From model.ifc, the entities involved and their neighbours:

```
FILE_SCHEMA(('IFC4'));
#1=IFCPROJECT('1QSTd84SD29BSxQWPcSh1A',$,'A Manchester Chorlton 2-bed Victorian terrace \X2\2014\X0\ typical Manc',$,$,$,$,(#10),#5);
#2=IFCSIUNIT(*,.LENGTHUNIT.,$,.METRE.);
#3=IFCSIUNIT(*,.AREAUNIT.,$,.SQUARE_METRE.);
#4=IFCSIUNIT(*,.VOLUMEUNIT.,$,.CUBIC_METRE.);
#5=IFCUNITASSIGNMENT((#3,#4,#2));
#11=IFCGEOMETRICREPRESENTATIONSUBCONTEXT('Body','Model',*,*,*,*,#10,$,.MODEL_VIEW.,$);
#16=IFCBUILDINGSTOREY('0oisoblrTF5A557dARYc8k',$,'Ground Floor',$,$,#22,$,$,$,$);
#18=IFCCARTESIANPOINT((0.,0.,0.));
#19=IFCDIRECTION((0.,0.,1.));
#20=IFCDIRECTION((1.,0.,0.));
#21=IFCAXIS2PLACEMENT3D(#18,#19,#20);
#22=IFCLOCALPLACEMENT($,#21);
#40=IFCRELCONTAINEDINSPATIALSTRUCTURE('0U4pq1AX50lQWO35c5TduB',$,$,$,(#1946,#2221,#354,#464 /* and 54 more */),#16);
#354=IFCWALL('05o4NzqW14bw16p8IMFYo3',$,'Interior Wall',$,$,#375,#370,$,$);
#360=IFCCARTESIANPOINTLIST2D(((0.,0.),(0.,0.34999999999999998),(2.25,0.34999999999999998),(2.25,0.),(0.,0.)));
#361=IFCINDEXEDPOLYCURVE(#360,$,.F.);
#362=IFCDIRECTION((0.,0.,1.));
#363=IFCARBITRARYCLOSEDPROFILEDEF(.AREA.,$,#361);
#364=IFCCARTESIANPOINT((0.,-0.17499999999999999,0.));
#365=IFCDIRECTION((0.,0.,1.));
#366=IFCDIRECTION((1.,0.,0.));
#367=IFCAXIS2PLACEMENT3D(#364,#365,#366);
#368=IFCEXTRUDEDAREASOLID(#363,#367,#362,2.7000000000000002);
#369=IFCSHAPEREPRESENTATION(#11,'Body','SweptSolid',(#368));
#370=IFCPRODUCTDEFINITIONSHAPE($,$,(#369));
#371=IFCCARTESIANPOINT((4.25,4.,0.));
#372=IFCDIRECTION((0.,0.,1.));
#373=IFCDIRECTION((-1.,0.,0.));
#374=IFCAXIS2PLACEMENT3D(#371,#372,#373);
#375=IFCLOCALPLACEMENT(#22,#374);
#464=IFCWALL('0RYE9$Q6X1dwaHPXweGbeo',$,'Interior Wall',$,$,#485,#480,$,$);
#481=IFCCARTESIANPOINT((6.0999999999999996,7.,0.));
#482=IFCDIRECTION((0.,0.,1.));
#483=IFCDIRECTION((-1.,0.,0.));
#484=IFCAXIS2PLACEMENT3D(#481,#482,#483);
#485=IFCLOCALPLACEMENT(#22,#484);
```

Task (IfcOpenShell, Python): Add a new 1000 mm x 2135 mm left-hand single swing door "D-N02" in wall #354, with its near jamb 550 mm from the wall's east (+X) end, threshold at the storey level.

```python
import numpy as np
import ifcopenshell
import ifcopenshell.api.feature
import ifcopenshell.api.geometry
import ifcopenshell.api.root
import ifcopenshell.api.spatial
import ifcopenshell.geom
import ifcopenshell.util.element
import ifcopenshell.util.placement
import ifcopenshell.util.representation
import ifcopenshell.util.shape
import ifcopenshell.util.unit

model = ifcopenshell.open("model.ifc")
unit_scale = ifcopenshell.util.unit.calculate_unit_scale(model)
settings = ifcopenshell.geom.settings()


def volume(element):
    """Net volume in cubic metres, openings subtracted."""
    shape = ifcopenshell.geom.create_shape(settings, element)
    return ifcopenshell.util.shape.get_volume(shape.geometry)


wall = model.by_id(354)
storey = ifcopenshell.util.element.get_container(wall, ifc_class="IfcBuildingStorey")
context = ifcopenshell.util.representation.get_context(model, "Model", "Body", "MODEL_VIEW")
before = volume(wall)

width, height, from_end, sill = 1, 2.135, 0.55, 0.0  # metres

# The wall runs along its own X axis, and the end named is its -X end.
wall_shape = ifcopenshell.geom.create_shape(settings, wall)
x, y, z = ifcopenshell.util.shape.get_vertices(wall_shape.geometry).T
start = x.min() + from_end
face, thickness = float(y.min()), float(y.max() - y.min())
wall_matrix = ifcopenshell.util.placement.get_local_placement(wall.ObjectPlacement)
level = ifcopenshell.util.placement.get_local_placement(storey.ObjectPlacement)[2, 3]


def in_wall(x, y):
    """Placement at x, y metres in the wall's axes, at sill height."""
    matrix = wall_matrix.copy()
    matrix[:, 3] = wall_matrix @ np.array([x / unit_scale, y / unit_scale, 0.0, 1.0])
    matrix[2, 3] = level + sill / unit_scale
    return matrix


# Opening: a box that overshoots both wall faces by 50 mm.
opening = ifcopenshell.api.root.create_entity(model, ifc_class="IfcOpeningElement", predefined_type="OPENING")
box = ifcopenshell.api.geometry.add_wall_representation(
    model, context=context, length=width, height=height, thickness=thickness + 0.1
)
ifcopenshell.api.geometry.assign_representation(model, product=opening, representation=box)
ifcopenshell.api.geometry.edit_object_placement(model, product=opening, matrix=in_wall(start, face - 0.05), is_si=False)
ifcopenshell.api.feature.add_feature(model, feature=opening, element=wall)

door = ifcopenshell.api.root.create_entity(model, ifc_class="IfcDoor", name="D-N02", predefined_type="DOOR")
door.OverallWidth, door.OverallHeight = width / unit_scale, height / unit_scale
door.OperationType = "SINGLE_SWING_LEFT"
body = ifcopenshell.api.geometry.add_door_representation(
    model,
    context=context,
    overall_width=door.OverallWidth,
    overall_height=door.OverallHeight,
    operation_type="SINGLE_SWING_LEFT",
    lining_properties={"LiningDepth": thickness / unit_scale, "ThresholdDepth": thickness / unit_scale},
)
ifcopenshell.api.geometry.assign_representation(model, product=door, representation=body)
ifcopenshell.api.spatial.assign_container(model, products=[door], relating_structure=storey)
ifcopenshell.api.feature.add_filling(model, opening=opening, element=door)

# The lining spans the wall, so the door starts at the wall face.
ifcopenshell.api.geometry.edit_object_placement(model, product=door, matrix=in_wall(start, face), is_si=False)

after = volume(wall)

print(f"wall volume {before:.3f} -> {after:.3f} m3")

model.write("model_v2.ifc")
```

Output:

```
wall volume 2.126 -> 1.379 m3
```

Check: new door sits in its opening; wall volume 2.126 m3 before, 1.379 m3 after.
